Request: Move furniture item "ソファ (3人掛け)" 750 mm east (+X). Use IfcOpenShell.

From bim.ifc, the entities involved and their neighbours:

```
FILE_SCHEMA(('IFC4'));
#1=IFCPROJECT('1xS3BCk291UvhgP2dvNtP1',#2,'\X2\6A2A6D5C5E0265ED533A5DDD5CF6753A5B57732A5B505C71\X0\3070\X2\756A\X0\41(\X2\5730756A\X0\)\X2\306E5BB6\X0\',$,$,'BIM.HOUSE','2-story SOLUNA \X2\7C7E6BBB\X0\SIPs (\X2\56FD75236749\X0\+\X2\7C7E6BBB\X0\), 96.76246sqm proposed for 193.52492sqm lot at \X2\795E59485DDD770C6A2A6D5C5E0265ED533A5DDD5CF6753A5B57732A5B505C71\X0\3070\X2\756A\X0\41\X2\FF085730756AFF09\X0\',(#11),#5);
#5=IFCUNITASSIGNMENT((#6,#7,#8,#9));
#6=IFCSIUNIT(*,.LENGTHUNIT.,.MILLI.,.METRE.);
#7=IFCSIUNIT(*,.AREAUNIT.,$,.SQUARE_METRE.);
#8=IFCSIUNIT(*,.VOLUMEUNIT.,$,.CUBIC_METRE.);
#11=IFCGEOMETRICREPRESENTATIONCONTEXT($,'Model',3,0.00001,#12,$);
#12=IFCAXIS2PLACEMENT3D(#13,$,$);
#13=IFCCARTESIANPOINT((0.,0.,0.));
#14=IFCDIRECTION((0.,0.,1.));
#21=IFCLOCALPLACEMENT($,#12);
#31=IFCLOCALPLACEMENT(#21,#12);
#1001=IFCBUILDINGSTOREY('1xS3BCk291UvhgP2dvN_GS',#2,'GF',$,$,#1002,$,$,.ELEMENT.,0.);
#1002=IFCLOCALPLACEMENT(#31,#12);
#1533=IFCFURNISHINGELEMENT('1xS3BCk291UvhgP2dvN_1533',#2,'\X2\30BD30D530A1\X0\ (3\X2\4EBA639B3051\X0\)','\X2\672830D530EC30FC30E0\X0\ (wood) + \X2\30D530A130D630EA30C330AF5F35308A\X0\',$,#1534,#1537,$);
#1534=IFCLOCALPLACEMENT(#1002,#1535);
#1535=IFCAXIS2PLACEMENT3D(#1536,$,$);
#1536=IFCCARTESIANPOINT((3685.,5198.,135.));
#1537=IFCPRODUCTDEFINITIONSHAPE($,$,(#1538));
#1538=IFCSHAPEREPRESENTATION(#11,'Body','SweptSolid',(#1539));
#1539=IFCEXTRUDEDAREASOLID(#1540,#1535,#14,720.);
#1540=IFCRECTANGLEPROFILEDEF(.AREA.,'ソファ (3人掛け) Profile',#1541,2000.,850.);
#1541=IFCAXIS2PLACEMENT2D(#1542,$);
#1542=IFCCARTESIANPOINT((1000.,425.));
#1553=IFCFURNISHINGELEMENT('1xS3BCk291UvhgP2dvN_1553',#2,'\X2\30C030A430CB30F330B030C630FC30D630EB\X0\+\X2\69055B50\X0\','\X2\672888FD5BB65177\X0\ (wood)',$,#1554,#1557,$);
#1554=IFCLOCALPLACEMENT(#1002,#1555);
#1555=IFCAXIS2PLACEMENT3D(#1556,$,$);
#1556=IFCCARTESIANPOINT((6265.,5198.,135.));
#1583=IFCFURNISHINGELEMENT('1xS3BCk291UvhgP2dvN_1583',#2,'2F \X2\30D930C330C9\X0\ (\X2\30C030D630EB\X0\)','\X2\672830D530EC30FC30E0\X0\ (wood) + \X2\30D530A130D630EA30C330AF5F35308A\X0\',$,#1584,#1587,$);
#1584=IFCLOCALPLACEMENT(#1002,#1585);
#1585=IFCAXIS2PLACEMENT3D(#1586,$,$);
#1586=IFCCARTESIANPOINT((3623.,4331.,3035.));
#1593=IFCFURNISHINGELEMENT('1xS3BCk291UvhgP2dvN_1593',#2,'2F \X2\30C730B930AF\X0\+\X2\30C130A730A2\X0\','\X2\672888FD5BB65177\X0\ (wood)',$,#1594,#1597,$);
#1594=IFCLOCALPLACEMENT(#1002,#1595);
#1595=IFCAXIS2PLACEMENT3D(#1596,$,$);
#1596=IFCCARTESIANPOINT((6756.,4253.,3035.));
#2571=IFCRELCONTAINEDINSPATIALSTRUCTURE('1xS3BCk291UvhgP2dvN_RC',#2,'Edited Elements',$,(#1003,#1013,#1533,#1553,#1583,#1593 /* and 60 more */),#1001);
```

```python
import ifcopenshell
import ifcopenshell.api.geometry
import ifcopenshell.util.placement
import ifcopenshell.util.unit

model = ifcopenshell.open("bim.ifc")
unit_scale = ifcopenshell.util.unit.calculate_unit_scale(model)

item = model.by_id(1533)
matrix = ifcopenshell.util.placement.get_local_placement(item.ObjectPlacement)
matrix[0, 3] += 0.75 / unit_scale
ifcopenshell.api.geometry.edit_object_placement(model, product=item, matrix=matrix, is_si=False)

print(ifcopenshell.util.placement.get_local_placement(item.ObjectPlacement).round(3) + 0.0)

model.write("bim_rev.ifc")
```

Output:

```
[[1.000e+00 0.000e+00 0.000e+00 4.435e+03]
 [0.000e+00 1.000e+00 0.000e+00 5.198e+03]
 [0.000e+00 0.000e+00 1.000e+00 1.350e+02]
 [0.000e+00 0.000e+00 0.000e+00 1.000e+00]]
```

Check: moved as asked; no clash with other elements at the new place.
